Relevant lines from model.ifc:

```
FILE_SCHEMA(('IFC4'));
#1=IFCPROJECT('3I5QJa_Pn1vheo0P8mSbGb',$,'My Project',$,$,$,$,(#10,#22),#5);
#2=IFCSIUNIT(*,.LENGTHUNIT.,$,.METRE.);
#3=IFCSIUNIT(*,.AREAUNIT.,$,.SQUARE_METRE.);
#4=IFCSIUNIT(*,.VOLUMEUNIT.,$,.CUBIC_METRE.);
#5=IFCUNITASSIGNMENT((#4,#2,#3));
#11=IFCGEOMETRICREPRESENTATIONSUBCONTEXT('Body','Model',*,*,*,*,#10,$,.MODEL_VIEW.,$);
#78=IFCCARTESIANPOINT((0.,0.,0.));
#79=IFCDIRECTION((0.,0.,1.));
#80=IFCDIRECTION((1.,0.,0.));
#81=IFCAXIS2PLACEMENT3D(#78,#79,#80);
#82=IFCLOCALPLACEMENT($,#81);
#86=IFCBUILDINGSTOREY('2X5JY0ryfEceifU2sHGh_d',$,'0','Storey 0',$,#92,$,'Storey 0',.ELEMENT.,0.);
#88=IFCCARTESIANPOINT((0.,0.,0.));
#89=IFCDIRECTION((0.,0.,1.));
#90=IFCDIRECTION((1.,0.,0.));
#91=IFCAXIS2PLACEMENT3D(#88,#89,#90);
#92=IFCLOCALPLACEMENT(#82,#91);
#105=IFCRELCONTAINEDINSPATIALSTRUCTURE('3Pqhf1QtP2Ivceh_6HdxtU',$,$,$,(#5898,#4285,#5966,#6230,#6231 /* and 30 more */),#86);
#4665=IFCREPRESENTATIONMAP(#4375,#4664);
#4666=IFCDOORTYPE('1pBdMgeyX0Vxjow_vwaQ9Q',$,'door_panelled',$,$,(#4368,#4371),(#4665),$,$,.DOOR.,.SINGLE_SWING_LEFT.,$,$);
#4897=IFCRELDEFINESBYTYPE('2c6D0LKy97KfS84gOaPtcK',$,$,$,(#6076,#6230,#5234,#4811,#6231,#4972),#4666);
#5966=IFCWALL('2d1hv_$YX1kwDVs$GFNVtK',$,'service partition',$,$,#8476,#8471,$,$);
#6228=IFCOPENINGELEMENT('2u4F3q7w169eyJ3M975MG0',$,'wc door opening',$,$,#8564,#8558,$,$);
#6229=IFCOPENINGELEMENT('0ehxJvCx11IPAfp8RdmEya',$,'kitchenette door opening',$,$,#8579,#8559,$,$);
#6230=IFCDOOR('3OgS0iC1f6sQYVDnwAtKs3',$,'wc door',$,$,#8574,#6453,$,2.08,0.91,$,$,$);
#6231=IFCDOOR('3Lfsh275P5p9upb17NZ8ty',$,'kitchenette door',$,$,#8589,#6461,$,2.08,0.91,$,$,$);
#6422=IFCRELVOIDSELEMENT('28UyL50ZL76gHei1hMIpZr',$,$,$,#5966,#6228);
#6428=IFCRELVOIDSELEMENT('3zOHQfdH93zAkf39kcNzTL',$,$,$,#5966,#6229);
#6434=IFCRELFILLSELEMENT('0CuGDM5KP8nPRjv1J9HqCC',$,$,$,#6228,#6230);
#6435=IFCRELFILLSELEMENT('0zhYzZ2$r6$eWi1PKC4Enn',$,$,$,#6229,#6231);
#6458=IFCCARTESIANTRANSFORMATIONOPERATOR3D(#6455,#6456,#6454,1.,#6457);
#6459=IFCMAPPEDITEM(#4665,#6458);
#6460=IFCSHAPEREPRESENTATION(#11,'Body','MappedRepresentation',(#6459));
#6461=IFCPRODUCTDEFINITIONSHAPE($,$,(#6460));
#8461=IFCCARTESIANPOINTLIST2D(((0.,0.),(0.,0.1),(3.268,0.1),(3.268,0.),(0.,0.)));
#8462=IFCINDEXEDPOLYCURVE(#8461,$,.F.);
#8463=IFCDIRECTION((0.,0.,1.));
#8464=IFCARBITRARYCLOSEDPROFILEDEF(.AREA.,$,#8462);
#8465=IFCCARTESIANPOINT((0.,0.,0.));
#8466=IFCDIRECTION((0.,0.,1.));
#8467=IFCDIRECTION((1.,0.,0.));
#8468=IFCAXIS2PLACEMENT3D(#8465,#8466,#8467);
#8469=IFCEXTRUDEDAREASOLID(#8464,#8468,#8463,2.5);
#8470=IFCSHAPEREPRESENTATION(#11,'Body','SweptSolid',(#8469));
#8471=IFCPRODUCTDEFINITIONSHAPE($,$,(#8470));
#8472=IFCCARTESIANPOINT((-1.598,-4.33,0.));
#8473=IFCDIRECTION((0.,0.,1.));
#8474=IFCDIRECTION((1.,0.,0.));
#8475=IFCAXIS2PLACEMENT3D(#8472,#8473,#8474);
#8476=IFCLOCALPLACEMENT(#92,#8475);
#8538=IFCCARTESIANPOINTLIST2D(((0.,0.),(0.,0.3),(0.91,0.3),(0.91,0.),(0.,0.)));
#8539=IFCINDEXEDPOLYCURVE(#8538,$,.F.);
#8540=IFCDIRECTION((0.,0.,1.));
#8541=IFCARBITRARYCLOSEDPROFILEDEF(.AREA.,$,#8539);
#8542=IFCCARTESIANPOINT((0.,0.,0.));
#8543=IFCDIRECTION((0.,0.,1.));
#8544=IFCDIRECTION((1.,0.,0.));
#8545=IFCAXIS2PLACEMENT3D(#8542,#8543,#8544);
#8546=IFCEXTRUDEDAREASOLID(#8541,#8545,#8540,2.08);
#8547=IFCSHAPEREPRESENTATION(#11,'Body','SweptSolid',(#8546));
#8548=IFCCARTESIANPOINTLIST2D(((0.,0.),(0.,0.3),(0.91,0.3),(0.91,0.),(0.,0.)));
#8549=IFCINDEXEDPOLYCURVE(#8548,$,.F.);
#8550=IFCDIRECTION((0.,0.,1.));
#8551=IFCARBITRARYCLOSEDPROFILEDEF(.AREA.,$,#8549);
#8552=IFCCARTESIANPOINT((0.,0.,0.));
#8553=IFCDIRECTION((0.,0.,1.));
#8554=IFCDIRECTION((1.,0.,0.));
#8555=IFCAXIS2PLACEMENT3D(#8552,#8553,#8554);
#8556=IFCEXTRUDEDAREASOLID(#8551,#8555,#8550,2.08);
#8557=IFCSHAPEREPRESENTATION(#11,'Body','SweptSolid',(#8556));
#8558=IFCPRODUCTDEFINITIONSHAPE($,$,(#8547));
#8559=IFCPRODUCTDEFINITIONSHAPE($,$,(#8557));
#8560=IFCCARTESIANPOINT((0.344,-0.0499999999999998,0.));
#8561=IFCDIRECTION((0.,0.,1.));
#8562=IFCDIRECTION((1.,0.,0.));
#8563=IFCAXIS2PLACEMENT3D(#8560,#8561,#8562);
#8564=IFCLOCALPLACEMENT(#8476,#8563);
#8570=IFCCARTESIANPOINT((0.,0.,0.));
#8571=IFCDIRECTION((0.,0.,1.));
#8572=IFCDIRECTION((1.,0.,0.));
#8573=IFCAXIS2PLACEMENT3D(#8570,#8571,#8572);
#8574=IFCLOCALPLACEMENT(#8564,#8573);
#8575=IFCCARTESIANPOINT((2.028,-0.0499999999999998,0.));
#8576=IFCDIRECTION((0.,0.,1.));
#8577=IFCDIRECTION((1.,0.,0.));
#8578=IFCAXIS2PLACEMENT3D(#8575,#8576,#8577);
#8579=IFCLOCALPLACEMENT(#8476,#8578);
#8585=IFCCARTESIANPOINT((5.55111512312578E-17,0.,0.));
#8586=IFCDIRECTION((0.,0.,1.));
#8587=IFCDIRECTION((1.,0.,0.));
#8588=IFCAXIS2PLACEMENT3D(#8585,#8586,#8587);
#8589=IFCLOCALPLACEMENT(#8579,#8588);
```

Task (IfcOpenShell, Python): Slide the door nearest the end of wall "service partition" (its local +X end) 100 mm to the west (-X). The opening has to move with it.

```python
import ifcopenshell
import ifcopenshell.api.geometry
import ifcopenshell.util.placement
import ifcopenshell.util.unit

model = ifcopenshell.open("model.ifc")
unit_scale = ifcopenshell.util.unit.calculate_unit_scale(model)

door = model.by_guid("3Lfsh275P5p9upb17NZ8ty")
opening = door.FillsVoids[0].RelatingOpeningElement
wall = opening.VoidsElements[0].RelatingBuildingElement

wall_matrix = ifcopenshell.util.placement.get_local_placement(wall.ObjectPlacement)
shift = wall_matrix[:3, 0] * -0.1 / unit_scale
before = ifcopenshell.util.placement.get_local_placement(door.ObjectPlacement)[:3, 3].copy()

# The door is placed relative to its opening, so it follows when the opening moves.
matrix = ifcopenshell.util.placement.get_local_placement(opening.ObjectPlacement)
matrix[:3, 3] += shift
ifcopenshell.api.geometry.edit_object_placement(
    model, product=opening, matrix=matrix, is_si=False, should_transform_children=True
)

after = ifcopenshell.util.placement.get_local_placement(door.ObjectPlacement)[:3, 3]
print("door moved by", (after - before).round(3) + 0.0)

model.write("model_rev.ifc")
```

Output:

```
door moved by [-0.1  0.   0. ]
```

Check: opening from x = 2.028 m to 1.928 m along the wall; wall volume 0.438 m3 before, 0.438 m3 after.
